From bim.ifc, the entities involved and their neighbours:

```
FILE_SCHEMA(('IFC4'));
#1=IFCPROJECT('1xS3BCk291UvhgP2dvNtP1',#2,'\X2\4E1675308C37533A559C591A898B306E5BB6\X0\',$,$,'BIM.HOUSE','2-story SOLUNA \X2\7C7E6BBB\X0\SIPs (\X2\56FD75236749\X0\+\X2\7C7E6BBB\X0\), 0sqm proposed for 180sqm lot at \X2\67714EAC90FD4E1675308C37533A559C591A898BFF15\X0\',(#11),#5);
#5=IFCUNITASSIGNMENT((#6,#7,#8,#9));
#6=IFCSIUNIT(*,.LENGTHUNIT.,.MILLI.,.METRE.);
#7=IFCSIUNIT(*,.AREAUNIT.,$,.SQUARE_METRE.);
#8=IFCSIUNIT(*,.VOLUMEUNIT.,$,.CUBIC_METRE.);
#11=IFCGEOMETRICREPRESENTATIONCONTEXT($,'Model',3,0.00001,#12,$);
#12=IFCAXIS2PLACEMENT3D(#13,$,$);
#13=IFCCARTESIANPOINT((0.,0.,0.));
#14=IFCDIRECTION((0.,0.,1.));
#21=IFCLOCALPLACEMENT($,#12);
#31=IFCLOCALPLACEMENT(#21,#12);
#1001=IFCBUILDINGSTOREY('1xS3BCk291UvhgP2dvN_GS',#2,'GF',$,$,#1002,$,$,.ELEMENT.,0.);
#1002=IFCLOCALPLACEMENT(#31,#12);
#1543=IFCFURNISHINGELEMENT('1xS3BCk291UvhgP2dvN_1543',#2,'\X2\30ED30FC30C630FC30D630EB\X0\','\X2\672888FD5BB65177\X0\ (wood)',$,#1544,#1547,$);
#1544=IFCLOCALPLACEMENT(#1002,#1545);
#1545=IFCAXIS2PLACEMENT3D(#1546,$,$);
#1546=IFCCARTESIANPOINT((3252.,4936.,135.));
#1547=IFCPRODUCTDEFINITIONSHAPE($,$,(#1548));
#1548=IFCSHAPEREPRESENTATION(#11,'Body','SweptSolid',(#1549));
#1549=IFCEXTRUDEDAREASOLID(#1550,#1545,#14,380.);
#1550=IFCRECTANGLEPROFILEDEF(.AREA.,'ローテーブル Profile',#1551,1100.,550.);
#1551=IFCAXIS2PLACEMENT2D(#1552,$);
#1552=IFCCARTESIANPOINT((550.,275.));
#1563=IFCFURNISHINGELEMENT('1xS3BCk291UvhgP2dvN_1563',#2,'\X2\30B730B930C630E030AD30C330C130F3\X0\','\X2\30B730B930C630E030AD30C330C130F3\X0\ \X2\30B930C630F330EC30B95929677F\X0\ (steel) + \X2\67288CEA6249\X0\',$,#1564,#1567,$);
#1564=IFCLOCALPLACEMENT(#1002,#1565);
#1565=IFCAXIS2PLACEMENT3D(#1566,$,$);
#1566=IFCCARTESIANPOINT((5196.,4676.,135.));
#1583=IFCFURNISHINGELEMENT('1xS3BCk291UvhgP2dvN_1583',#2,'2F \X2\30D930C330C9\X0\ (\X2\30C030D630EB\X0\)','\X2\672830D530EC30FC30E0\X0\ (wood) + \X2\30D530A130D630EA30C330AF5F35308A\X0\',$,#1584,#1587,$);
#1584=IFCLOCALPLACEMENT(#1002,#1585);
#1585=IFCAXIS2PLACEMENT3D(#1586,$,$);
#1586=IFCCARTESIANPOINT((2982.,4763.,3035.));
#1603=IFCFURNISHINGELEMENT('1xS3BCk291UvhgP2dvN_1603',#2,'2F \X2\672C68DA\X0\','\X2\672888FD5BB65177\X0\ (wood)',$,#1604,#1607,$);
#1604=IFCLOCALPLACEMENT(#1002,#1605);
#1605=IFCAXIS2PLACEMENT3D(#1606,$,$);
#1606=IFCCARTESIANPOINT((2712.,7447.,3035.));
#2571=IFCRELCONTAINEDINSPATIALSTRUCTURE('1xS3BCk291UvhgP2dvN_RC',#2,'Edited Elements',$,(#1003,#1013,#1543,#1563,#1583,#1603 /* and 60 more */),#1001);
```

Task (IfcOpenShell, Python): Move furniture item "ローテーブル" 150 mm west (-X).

```python
import ifcopenshell
import ifcopenshell.api.geometry
import ifcopenshell.util.placement

model = ifcopenshell.open("bim.ifc")

item = model.by_guid("1xS3BCk291UvhgP2dvN_1543")
matrix = ifcopenshell.util.placement.get_local_placement(item.ObjectPlacement)
matrix[0, 3] -= 150.0
ifcopenshell.api.geometry.edit_object_placement(model, product=item, matrix=matrix, is_si=False)

print(ifcopenshell.util.placement.get_local_placement(item.ObjectPlacement).round(3) + 0.0)

model.write("bim_edited.ifc")
```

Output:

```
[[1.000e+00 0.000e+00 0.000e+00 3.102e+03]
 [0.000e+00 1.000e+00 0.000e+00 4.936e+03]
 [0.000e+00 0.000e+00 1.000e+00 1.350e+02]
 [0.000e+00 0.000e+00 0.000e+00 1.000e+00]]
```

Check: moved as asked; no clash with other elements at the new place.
